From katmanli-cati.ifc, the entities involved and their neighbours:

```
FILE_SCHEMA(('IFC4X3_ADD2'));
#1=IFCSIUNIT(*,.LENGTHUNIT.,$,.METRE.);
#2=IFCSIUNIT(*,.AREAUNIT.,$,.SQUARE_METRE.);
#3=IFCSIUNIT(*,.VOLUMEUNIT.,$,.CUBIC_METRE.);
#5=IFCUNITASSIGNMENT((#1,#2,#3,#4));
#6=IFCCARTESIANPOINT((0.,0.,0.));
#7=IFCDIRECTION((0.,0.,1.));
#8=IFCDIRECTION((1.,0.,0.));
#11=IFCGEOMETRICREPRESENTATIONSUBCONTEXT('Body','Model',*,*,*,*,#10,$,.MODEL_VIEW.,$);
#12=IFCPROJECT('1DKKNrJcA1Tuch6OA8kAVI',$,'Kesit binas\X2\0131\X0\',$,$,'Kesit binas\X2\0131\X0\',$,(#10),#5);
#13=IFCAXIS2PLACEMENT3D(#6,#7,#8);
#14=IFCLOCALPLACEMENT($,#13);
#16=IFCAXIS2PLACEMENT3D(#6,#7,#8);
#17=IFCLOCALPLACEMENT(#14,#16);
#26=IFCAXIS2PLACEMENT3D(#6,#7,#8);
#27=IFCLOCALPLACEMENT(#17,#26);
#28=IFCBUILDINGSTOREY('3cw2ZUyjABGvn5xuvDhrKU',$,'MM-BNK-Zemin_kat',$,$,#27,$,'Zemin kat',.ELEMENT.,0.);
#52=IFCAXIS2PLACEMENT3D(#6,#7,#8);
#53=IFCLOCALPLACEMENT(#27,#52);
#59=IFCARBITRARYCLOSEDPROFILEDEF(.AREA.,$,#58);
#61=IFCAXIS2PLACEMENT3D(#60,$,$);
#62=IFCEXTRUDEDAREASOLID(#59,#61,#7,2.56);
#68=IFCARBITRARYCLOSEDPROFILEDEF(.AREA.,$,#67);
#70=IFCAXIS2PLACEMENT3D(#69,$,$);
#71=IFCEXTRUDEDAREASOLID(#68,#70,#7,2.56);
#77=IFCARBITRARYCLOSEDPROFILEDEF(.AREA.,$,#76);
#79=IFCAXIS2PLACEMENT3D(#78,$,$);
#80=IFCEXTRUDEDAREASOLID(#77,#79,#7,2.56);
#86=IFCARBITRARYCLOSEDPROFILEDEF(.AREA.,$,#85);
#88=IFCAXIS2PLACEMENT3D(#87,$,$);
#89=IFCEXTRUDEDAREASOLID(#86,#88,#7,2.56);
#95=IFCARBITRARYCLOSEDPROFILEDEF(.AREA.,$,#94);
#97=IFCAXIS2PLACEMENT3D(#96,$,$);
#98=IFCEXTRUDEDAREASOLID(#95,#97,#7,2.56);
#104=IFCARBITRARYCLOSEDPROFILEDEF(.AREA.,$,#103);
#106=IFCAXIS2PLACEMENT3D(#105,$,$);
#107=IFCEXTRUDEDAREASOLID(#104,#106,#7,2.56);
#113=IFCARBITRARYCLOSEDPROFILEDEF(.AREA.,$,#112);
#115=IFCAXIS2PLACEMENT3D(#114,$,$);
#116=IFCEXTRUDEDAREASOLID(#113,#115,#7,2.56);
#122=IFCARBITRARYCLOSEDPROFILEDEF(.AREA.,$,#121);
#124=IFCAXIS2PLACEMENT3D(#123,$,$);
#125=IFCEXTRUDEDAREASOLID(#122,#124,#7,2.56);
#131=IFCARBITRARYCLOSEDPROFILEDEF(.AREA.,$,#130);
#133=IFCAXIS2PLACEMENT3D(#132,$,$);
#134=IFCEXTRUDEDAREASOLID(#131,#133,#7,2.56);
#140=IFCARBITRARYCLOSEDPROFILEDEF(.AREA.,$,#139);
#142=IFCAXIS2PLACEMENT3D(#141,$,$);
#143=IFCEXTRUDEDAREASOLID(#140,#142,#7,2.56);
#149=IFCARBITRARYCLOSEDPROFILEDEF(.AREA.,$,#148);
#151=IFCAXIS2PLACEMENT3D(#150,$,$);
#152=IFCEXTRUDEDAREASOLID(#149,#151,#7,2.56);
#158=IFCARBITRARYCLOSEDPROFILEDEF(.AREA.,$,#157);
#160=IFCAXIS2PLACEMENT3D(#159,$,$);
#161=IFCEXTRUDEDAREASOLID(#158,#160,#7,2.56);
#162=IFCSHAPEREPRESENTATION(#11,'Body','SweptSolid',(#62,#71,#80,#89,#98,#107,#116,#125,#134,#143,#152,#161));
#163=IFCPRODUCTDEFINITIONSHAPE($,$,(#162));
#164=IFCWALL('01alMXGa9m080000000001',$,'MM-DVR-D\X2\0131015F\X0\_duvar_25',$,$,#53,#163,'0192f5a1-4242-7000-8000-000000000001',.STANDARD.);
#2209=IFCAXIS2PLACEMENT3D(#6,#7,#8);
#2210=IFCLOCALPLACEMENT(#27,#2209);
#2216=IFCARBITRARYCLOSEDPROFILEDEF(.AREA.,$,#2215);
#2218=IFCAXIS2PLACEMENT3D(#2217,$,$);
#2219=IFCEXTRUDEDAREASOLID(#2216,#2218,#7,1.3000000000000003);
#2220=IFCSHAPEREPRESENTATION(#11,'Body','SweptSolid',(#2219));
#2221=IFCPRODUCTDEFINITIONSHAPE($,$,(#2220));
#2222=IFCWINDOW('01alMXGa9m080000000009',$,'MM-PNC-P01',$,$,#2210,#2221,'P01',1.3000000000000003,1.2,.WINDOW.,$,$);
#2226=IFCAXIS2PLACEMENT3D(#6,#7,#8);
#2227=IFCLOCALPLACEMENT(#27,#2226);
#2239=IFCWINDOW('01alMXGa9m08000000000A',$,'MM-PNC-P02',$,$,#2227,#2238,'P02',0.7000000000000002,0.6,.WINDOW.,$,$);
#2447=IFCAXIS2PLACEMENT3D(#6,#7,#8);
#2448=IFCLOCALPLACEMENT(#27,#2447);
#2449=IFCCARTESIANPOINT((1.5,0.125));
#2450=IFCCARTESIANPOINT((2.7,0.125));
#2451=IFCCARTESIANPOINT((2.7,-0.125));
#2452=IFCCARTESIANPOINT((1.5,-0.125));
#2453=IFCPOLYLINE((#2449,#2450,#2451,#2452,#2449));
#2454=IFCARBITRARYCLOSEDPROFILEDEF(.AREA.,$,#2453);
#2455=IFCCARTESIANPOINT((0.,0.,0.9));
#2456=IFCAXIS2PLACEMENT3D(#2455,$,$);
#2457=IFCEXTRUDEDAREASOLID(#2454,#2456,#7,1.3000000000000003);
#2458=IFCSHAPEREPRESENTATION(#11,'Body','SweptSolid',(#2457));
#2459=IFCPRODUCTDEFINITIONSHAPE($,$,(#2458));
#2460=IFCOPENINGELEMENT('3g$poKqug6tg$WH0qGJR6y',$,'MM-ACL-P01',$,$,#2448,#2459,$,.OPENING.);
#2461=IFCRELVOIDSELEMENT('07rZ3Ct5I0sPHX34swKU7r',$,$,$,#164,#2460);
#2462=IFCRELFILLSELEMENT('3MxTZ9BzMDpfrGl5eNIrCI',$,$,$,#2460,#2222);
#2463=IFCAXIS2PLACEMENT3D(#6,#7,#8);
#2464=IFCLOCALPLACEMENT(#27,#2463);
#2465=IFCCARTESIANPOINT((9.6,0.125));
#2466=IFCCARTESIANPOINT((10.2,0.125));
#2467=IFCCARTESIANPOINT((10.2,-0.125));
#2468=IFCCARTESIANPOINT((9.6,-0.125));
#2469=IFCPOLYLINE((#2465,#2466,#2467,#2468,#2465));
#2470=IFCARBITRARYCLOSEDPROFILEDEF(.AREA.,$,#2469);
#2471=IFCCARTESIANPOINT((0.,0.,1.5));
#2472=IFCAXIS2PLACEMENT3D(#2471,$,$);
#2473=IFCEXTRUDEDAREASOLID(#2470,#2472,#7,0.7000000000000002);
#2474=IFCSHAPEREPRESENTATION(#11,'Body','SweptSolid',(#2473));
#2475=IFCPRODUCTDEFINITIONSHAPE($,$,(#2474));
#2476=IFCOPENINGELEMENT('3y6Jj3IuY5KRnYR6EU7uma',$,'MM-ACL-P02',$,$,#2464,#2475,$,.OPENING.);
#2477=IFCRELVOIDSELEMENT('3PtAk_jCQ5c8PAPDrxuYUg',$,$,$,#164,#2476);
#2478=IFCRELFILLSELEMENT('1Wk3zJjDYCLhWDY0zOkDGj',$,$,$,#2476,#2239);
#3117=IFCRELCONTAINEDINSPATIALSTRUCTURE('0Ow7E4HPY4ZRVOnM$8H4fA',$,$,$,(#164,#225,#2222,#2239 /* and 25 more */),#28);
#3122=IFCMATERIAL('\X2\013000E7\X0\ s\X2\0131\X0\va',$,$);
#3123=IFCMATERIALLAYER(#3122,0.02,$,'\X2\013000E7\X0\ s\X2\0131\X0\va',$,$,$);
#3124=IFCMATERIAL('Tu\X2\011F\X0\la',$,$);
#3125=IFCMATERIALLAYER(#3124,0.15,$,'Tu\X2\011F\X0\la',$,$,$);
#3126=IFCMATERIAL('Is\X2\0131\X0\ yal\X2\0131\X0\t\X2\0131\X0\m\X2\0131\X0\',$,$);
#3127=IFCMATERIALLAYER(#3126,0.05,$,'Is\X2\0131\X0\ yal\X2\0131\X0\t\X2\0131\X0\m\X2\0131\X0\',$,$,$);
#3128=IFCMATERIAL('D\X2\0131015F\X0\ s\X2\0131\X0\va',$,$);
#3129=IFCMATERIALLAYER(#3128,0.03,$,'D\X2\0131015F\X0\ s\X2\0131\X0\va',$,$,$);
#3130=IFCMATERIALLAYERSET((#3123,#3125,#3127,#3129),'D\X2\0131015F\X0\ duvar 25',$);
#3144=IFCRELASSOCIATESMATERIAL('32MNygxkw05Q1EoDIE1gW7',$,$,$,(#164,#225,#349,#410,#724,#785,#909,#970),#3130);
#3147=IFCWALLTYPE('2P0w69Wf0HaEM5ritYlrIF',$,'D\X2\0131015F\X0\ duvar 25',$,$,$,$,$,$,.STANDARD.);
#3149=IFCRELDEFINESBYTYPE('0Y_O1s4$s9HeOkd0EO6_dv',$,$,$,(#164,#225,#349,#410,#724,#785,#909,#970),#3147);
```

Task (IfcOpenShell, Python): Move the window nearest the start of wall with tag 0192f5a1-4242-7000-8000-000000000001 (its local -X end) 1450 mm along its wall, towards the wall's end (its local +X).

```python
import ifcopenshell
import ifcopenshell.api.geometry
import ifcopenshell.util.placement
import ifcopenshell.util.unit

model = ifcopenshell.open("katmanli-cati.ifc")
unit_scale = ifcopenshell.util.unit.calculate_unit_scale(model)

window = model.by_guid("01alMXGa9m080000000009")
opening = window.FillsVoids[0].RelatingOpeningElement
wall = opening.VoidsElements[0].RelatingBuildingElement

wall_matrix = ifcopenshell.util.placement.get_local_placement(wall.ObjectPlacement)
shift = wall_matrix[:3, 0] * 1.45 / unit_scale
before = ifcopenshell.util.placement.get_local_placement(window.ObjectPlacement)[:3, 3].copy()

# The window is not placed relative to its opening, so move both.
for product in (opening, window):
    matrix = ifcopenshell.util.placement.get_local_placement(product.ObjectPlacement)
    matrix[:3, 3] += shift
    ifcopenshell.api.geometry.edit_object_placement(model, product=product, matrix=matrix, is_si=False)

after = ifcopenshell.util.placement.get_local_placement(window.ObjectPlacement)[:3, 3]
print("window moved by", (after - before).round(3) + 0.0)

model.write("katmanli-cati_rev.ifc")
```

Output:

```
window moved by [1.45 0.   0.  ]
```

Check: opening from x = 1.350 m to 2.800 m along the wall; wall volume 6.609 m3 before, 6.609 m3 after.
